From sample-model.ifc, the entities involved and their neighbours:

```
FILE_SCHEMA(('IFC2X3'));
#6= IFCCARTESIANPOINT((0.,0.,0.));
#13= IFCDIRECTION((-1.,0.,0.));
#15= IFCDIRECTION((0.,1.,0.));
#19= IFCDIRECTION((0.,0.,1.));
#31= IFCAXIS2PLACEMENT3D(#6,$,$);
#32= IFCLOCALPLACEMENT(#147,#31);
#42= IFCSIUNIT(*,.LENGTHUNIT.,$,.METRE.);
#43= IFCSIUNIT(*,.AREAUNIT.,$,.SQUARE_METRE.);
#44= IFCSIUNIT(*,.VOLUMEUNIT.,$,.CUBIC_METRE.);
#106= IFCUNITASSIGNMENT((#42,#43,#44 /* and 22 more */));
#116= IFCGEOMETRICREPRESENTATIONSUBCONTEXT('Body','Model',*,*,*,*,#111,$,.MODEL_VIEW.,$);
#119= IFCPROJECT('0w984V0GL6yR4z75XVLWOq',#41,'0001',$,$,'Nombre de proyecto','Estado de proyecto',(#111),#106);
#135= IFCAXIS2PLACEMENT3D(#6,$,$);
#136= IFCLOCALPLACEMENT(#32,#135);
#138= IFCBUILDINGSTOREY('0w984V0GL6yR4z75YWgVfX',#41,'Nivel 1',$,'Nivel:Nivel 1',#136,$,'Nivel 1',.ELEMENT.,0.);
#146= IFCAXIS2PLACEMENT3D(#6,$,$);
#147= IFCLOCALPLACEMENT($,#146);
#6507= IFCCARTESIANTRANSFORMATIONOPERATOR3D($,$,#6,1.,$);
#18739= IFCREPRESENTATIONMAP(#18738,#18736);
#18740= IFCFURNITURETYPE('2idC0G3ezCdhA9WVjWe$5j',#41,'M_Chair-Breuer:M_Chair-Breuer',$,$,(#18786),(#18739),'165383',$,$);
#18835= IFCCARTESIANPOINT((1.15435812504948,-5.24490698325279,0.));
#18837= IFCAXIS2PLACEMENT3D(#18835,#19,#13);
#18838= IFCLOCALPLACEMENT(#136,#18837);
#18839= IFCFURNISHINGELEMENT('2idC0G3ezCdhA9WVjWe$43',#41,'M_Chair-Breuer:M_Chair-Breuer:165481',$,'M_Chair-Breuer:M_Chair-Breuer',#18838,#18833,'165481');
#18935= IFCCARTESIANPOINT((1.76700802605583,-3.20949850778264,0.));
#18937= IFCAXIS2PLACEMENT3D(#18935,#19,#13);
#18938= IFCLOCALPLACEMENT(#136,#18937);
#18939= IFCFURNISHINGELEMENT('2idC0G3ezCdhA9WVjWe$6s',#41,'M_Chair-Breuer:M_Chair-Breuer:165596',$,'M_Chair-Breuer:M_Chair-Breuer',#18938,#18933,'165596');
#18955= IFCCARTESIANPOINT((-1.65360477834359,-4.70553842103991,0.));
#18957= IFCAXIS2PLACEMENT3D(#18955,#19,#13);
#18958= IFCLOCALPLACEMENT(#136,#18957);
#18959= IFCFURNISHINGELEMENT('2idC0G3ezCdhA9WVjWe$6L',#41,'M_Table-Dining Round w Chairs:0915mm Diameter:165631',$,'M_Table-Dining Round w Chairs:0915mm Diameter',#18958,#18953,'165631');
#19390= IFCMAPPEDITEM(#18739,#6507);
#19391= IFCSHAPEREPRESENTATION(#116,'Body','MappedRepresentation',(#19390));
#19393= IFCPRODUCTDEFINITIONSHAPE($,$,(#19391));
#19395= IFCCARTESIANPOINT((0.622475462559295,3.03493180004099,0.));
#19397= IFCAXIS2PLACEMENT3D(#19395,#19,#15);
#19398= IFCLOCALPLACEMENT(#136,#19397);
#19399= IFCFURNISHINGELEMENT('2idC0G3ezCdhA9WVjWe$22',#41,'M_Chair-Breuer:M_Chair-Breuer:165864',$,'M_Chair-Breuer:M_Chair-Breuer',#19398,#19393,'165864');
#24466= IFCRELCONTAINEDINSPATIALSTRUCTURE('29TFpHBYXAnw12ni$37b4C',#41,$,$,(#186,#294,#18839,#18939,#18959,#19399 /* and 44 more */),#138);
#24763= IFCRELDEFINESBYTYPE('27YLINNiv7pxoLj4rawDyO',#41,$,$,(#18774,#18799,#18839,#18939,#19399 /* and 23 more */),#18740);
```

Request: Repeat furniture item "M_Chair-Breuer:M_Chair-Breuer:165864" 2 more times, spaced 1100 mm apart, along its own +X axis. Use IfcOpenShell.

```python
import ifcopenshell
import ifcopenshell.api.geometry
import ifcopenshell.api.root
import ifcopenshell.util.element
import ifcopenshell.util.placement
import ifcopenshell.util.unit

model = ifcopenshell.open("sample-model.ifc")
unit_scale = ifcopenshell.util.unit.calculate_unit_scale(model)


def reuse_history(source, copy):
    """copy_class also copies each property set's owner history, people and application; keep the originals."""
    for rel in copy.IsDefinedBy:
        if rel.is_a("IfcRelDefinesByProperties") and (history := rel.RelatingPropertyDefinition.OwnerHistory):
            rel.RelatingPropertyDefinition.OwnerHistory = source.OwnerHistory
            ifcopenshell.util.element.remove_deep2(model, history)


source = model.by_guid("2idC0G3ezCdhA9WVjWe$22")
base = ifcopenshell.util.placement.get_local_placement(source.ObjectPlacement)
step = base[:3, 0] * 1.1 / unit_scale

for i in range(1, 3):
    copy = ifcopenshell.api.root.copy_class(model, product=source)
    copy.Representation = ifcopenshell.util.element.copy_deep(
        model, source.Representation, exclude=["IfcGeometricRepresentationContext", "IfcRepresentationMap"]
    )
    copy.Name = "M_Chair-Breuer:M_Chair-Breuer"
    copy.Tag = None
    reuse_history(source, copy)
    matrix = base.copy()
    matrix[:3, 3] += i * step
    print("added at", matrix[:3, 3].round(3) + 0.0)
    ifcopenshell.api.geometry.edit_object_placement(model, product=copy, matrix=matrix, is_si=False)

model.write("sample-model_rev.ifc")
```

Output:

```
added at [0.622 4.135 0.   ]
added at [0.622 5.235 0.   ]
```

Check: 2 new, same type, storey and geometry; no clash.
